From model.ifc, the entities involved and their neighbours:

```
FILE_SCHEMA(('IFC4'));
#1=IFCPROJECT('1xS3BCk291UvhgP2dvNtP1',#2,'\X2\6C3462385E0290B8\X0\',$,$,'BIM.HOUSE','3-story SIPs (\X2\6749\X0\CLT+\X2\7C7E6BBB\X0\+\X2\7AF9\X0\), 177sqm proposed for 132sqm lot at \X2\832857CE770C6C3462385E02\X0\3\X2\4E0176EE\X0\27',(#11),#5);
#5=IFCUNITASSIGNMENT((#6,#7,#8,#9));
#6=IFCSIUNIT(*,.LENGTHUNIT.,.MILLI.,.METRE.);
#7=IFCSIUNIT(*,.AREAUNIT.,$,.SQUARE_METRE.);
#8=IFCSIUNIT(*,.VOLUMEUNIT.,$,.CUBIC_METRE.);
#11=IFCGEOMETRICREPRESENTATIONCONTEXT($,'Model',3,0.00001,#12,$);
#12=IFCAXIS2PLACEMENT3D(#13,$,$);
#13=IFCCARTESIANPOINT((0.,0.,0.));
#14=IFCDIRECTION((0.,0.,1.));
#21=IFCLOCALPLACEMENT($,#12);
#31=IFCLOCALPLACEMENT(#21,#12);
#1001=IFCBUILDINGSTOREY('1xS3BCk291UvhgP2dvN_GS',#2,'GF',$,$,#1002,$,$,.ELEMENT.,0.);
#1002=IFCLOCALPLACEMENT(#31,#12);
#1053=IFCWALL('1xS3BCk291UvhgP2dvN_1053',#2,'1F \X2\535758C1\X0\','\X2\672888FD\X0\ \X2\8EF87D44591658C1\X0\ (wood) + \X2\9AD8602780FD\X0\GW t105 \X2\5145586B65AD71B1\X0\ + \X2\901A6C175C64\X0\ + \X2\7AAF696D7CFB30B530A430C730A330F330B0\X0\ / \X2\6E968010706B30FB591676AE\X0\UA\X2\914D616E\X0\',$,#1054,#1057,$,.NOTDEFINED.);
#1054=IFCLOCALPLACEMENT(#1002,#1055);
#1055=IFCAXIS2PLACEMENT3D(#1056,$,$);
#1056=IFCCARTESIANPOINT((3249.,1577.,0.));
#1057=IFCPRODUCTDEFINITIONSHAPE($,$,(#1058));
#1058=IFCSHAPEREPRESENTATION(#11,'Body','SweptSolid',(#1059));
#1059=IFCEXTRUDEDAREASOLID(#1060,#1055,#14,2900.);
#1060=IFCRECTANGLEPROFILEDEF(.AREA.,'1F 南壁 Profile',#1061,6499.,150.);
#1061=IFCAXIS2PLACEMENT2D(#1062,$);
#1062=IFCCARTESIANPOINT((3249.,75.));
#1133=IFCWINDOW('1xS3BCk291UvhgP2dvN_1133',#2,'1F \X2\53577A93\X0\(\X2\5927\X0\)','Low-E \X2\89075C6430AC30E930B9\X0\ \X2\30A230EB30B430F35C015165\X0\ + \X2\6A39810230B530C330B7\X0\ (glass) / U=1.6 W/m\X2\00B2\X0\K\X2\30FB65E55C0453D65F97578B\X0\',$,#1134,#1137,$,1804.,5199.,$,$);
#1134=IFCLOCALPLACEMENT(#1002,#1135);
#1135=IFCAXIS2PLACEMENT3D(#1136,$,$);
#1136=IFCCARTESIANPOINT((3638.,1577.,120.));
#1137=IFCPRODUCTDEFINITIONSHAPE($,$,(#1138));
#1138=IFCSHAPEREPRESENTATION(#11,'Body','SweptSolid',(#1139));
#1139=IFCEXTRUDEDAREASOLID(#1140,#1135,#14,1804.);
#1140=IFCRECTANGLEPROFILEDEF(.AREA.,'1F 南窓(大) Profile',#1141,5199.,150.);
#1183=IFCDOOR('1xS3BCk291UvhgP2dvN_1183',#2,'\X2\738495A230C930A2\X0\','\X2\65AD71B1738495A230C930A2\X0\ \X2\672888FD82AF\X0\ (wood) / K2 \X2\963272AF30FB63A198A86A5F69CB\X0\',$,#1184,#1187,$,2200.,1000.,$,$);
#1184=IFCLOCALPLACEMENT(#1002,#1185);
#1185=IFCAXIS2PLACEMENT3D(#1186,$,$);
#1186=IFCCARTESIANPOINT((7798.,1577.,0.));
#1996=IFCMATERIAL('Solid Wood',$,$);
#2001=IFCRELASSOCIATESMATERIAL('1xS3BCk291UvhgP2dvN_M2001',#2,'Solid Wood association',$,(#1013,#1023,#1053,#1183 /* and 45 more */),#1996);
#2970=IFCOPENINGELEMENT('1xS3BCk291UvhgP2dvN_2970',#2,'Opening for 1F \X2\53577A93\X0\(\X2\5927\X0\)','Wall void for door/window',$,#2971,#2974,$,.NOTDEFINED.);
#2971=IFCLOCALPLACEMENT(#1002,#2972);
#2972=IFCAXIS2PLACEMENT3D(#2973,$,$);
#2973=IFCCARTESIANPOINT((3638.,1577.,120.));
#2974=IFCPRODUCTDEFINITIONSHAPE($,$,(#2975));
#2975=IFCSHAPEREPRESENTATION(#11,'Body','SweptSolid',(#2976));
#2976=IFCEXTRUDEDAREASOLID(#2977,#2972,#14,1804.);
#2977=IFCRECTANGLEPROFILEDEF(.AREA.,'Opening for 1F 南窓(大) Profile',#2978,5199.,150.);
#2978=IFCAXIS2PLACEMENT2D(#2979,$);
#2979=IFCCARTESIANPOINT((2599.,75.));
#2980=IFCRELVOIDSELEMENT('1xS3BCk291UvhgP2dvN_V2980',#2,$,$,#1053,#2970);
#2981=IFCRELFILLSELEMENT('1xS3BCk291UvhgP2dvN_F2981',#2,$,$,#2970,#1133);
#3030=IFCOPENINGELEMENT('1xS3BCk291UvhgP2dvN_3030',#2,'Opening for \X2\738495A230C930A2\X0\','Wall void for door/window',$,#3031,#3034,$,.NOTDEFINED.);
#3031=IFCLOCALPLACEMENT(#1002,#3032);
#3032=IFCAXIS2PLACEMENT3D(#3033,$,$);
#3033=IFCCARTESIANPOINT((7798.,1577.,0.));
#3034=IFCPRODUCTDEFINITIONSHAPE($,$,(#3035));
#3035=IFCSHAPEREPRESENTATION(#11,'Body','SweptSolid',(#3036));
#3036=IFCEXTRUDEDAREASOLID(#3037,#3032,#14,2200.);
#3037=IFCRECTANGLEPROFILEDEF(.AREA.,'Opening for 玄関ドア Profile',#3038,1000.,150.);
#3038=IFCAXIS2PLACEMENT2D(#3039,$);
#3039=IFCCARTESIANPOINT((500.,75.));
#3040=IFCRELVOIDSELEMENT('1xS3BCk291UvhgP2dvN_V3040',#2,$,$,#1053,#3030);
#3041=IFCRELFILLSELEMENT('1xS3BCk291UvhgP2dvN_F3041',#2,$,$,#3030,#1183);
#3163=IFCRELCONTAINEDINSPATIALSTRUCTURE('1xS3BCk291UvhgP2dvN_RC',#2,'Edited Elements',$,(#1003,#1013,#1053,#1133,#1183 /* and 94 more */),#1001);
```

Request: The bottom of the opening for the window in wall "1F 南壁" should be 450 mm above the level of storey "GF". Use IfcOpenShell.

```python
import numpy as np
import ifcopenshell
import ifcopenshell.api.geometry
import ifcopenshell.geom
import ifcopenshell.util.element
import ifcopenshell.util.placement
import ifcopenshell.util.shape
import ifcopenshell.util.unit

model = ifcopenshell.open("model.ifc")
unit_scale = ifcopenshell.util.unit.calculate_unit_scale(model)

window = model.by_guid("1xS3BCk291UvhgP2dvN_1133")
opening = window.FillsVoids[0].RelatingOpeningElement
storey = ifcopenshell.util.element.get_container(window, ifc_class="IfcBuildingStorey")
level = ifcopenshell.util.placement.get_local_placement(storey.ObjectPlacement)[2, 3]

# The opening's origin need not be at the sill, so measure its lowest point.
shape = ifcopenshell.geom.create_shape(ifcopenshell.geom.settings(), opening)
bottom = ifcopenshell.util.shape.get_shape_bottom_elevation(shape, shape.geometry) / unit_scale
dz = level + 0.45 / unit_scale - bottom

shift = np.array([0.0, 0.0, dz])
# The window is not placed relative to its opening, so move both.
for product in (opening, window):
    matrix = ifcopenshell.util.placement.get_local_placement(product.ObjectPlacement)
    matrix[:3, 3] += shift
    ifcopenshell.api.geometry.edit_object_placement(model, product=product, matrix=matrix, is_si=False)

print(f"moved by {dz * unit_scale:+.3f} m")

model.write("model_rev.ifc")
```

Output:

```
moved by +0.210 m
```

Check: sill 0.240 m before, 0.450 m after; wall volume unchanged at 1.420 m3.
